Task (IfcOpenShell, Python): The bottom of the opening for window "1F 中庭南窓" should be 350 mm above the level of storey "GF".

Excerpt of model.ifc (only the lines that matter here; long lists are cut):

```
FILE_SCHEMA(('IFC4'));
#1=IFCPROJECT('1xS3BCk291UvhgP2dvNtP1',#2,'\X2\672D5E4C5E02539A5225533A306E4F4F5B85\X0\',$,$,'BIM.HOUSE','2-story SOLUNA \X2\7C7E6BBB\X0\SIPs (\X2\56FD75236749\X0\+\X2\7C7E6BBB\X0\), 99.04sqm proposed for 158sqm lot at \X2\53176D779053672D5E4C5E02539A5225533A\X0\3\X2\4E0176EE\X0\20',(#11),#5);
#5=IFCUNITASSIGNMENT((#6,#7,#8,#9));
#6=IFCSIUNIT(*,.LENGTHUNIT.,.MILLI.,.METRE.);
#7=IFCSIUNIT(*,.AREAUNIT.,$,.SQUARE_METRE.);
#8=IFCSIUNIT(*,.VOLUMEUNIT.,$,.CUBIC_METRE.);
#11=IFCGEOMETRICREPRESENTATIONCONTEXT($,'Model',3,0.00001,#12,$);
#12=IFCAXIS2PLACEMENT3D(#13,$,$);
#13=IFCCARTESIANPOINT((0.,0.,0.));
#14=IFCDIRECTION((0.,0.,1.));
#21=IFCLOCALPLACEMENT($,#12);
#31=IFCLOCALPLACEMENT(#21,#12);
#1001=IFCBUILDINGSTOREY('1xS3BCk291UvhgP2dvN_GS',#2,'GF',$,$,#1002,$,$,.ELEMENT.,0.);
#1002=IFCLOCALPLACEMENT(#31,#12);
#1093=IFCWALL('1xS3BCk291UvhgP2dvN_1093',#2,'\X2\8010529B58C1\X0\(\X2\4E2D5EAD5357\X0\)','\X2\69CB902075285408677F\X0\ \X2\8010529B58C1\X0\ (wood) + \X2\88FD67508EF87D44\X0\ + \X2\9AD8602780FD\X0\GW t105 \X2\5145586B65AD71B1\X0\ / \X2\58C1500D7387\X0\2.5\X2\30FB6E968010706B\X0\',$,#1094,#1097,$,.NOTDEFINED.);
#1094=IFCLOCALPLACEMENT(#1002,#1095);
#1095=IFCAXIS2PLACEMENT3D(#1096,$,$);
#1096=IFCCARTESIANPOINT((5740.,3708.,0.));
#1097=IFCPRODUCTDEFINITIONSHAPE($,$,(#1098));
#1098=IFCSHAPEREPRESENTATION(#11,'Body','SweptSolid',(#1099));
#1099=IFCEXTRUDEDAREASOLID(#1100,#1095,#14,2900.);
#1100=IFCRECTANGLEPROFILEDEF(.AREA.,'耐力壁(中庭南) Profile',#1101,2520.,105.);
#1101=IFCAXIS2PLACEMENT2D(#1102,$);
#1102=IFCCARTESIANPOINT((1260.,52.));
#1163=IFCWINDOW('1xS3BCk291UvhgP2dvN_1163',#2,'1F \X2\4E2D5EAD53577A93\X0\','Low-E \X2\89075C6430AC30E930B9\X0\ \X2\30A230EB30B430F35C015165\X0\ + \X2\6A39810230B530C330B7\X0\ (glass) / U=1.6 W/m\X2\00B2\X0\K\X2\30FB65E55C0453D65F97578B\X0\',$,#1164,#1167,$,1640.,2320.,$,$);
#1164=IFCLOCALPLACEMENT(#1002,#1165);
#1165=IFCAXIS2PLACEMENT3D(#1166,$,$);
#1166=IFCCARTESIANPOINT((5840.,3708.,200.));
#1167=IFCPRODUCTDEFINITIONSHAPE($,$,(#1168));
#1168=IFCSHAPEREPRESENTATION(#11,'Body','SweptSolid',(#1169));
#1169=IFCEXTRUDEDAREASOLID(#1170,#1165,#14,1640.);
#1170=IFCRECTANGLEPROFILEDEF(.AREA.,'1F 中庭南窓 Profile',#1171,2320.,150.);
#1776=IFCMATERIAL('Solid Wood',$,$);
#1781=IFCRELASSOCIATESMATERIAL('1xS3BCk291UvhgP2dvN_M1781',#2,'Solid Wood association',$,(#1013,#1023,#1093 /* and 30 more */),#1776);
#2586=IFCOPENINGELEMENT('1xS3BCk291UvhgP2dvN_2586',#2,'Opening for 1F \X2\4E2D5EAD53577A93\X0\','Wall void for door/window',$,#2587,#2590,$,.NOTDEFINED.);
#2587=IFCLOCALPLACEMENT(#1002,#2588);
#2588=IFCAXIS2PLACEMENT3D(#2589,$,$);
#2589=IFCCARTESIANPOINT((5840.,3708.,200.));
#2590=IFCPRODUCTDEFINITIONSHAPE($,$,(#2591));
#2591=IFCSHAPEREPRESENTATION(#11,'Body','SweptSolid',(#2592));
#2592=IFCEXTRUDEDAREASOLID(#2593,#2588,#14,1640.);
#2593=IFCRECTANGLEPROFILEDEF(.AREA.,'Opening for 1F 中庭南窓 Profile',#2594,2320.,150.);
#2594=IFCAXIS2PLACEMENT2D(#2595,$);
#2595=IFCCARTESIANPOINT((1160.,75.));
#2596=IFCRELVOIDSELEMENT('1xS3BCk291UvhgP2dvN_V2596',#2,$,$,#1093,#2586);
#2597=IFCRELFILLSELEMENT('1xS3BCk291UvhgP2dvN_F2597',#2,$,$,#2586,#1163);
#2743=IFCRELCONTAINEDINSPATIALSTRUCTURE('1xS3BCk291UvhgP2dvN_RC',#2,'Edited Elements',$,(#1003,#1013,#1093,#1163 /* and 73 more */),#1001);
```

```python
import numpy as np
import ifcopenshell
import ifcopenshell.api.geometry
import ifcopenshell.geom
import ifcopenshell.util.element
import ifcopenshell.util.placement
import ifcopenshell.util.shape
import ifcopenshell.util.unit

model = ifcopenshell.open("model.ifc")
unit_scale = ifcopenshell.util.unit.calculate_unit_scale(model)

window = model.by_guid("1xS3BCk291UvhgP2dvN_1163")
opening = window.FillsVoids[0].RelatingOpeningElement
storey = ifcopenshell.util.element.get_container(window, ifc_class="IfcBuildingStorey")
level = ifcopenshell.util.placement.get_local_placement(storey.ObjectPlacement)[2, 3]

# The opening's origin need not be at the sill, so measure its lowest point.
shape = ifcopenshell.geom.create_shape(ifcopenshell.geom.settings(), opening)
bottom = ifcopenshell.util.shape.get_shape_bottom_elevation(shape, shape.geometry) / unit_scale
dz = level + 0.35 / unit_scale - bottom

shift = np.array([0.0, 0.0, dz])
# The window is not placed relative to its opening, so move both.
for product in (opening, window):
    matrix = ifcopenshell.util.placement.get_local_placement(product.ObjectPlacement)
    matrix[:3, 3] += shift
    ifcopenshell.api.geometry.edit_object_placement(model, product=product, matrix=matrix, is_si=False)

print(f"moved by {dz * unit_scale:+.3f} m")

model.write("model_edited.ifc")
```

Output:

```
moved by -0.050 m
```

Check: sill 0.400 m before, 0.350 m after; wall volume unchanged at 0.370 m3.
